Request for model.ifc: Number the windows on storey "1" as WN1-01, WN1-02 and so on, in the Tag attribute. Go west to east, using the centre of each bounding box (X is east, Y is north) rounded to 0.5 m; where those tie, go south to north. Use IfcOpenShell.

First a look at what the model holds.

```python
import ifcopenshell
import ifcopenshell.util.element
import ifcopenshell.util.placement

model = ifcopenshell.open("model.ifc")
print(model.schema)
storey = next(s for s in model.by_type("IfcBuildingStorey") if s.Name == "1")
windows = [e for e in ifcopenshell.util.element.get_decomposition(storey) if e.is_a("IfcWindow")]
for e in sorted(windows, key=lambda e: e.id()):
    origin = ifcopenshell.util.placement.get_local_placement(e.ObjectPlacement)[:3, 3]
    print(e.id(), e.Tag, e.Name, origin.round(2) + 0.0, sep=" | ")
```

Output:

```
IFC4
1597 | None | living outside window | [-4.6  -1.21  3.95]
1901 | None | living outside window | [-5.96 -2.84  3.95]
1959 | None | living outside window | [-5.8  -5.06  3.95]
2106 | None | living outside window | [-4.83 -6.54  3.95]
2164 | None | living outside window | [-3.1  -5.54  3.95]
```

```python
import ifcopenshell
import ifcopenshell.geom
import ifcopenshell.util.element
import ifcopenshell.util.shape

model = ifcopenshell.open("model.ifc")
settings = ifcopenshell.geom.settings()
settings.set("use-world-coords", True)


def centre(element):
    shape = ifcopenshell.geom.create_shape(settings, element)
    return ifcopenshell.util.shape.get_bbox_centroid(shape.geometry)


storey = next(s for s in model.by_type("IfcBuildingStorey") if s.Name == "1")
windows = [e for e in ifcopenshell.util.element.get_decomposition(storey) if e.is_a("IfcWindow")]

# Insertion points can sit at a corner or the storey origin, so sort by the geometry (in metres).
centres = {e: centre(e) for e in windows}
windows.sort(key=lambda e: (round(centres[e][0] / 0.5), centres[e][1]))

for i, e in enumerate(windows, start=1):
    number = f"WN1-{i:02d}"
    e.Tag = number
    print(e.id(), number)

model.write("model-out.ifc")
```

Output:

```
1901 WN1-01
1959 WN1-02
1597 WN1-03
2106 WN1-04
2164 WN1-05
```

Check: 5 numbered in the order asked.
